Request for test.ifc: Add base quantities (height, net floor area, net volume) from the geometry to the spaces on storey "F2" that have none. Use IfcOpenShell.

First a look at what the model holds.

```python
import ifcopenshell
import ifcopenshell.util.element
import ifcopenshell.util.unit

model = ifcopenshell.open("test.ifc")
print(model.schema)
for unit_type in ("LENGTHUNIT", "AREAUNIT", "VOLUMEUNIT"):
    print(unit_type, ifcopenshell.util.unit.calculate_unit_scale(model, unit_type))
storey = next(s for s in model.by_type("IfcBuildingStorey") if s.Name == "F2")
spaces = [e for e in ifcopenshell.util.element.get_decomposition(storey) if e.is_a("IfcSpace")]
for e in sorted(spaces, key=lambda e: e.id()):
    print(e.id(), e.is_a(), e.Name, list(ifcopenshell.util.element.get_psets(e, qtos_only=True)), sep=" | ")
```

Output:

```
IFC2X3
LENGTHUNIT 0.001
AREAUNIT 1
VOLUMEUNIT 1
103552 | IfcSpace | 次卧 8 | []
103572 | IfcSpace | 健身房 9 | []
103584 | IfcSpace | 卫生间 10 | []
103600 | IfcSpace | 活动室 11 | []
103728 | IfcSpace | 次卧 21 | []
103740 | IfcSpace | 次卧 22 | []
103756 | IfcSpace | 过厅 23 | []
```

```python
import ifcopenshell
import ifcopenshell.api.pset
import ifcopenshell.geom
import ifcopenshell.util.element
import ifcopenshell.util.shape
import ifcopenshell.util.unit

model = ifcopenshell.open("test.ifc")
unit_scale = ifcopenshell.util.unit.calculate_unit_scale(model)
area_scale = ifcopenshell.util.unit.calculate_unit_scale(model, "AREAUNIT")
volume_scale = ifcopenshell.util.unit.calculate_unit_scale(model, "VOLUMEUNIT")
settings = ifcopenshell.geom.settings()

storey = next(s for s in model.by_type("IfcBuildingStorey") if s.Name == "F2")
spaces = [e for e in ifcopenshell.util.element.get_decomposition(storey) if e.is_a("IfcSpace")]

for e in sorted(spaces, key=lambda e: e.id()):
    if ifcopenshell.util.element.get_psets(e, qtos_only=True, should_inherit=False):
        continue
    # Geometry comes back in metres, in the element's own axes.
    shape = ifcopenshell.geom.create_shape(settings, e)
    values = {
        "Height": ifcopenshell.util.shape.get_z(shape.geometry) / unit_scale,
        "NetFloorArea": ifcopenshell.util.shape.get_footprint_area(shape.geometry) / area_scale,
        "NetVolume": ifcopenshell.util.shape.get_volume(shape.geometry) / volume_scale,
    }
    qto = ifcopenshell.api.pset.add_qto(model, product=e, name="BaseQuantities")
    ifcopenshell.api.pset.edit_qto(model, qto=qto, properties=values)
    print(e.id(), {k: round(v, 3) for k, v in values.items()})

model.write("test_v2.ifc")
```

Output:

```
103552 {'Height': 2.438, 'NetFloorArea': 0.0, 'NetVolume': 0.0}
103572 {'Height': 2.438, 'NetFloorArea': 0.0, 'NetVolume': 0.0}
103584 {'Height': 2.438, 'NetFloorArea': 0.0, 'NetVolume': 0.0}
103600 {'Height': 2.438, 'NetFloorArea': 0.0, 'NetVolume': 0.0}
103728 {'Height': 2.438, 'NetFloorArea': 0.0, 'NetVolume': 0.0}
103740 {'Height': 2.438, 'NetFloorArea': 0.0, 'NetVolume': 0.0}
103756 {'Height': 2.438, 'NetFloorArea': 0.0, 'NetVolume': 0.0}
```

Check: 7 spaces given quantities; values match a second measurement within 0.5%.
